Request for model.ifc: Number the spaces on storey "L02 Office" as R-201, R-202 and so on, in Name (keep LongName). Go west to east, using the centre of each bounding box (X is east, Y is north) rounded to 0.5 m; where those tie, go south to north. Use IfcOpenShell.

First a look at what the model holds.

```python
import ifcopenshell
import ifcopenshell.util.element
import ifcopenshell.util.placement

model = ifcopenshell.open("model.ifc")
print(model.schema)
storey = next(s for s in model.by_type("IfcBuildingStorey") if s.Name == "L02 Office")
spaces = [e for e in ifcopenshell.util.element.get_decomposition(storey) if e.is_a("IfcSpace")]
for e in sorted(spaces, key=lambda e: e.id()):
    origin = ifcopenshell.util.placement.get_local_placement(e.ObjectPlacement)[:3, 3]
    print(e.id(), e.Name, e.LongName, origin.round(2) + 0.0, sep=" | ")
```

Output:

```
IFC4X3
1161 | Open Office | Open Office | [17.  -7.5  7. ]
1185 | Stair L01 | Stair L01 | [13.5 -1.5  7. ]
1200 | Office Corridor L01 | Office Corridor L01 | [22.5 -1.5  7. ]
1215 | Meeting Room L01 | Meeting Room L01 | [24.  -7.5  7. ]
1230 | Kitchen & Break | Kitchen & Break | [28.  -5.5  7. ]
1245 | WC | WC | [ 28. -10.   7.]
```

```python
import ifcopenshell
import ifcopenshell.geom
import ifcopenshell.util.element
import ifcopenshell.util.shape

model = ifcopenshell.open("model.ifc")
settings = ifcopenshell.geom.settings()
settings.set("use-world-coords", True)


def centre(element):
    shape = ifcopenshell.geom.create_shape(settings, element)
    return ifcopenshell.util.shape.get_bbox_centroid(shape.geometry)


storey = next(s for s in model.by_type("IfcBuildingStorey") if s.Name == "L02 Office")
spaces = [e for e in ifcopenshell.util.element.get_decomposition(storey) if e.is_a("IfcSpace")]

# Insertion points can sit at a corner or the storey origin, so sort by the geometry (in metres).
centres = {e: centre(e) for e in spaces}
spaces.sort(key=lambda e: (round(centres[e][0] / 0.5), centres[e][1]))

for i, e in enumerate(spaces, start=1):
    number = f"R-2{i:02d}"
    e.Name = number
    print(e.id(), number)

model.write("model_updated.ifc")
```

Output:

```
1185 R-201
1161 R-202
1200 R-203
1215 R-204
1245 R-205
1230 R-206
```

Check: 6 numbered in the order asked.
